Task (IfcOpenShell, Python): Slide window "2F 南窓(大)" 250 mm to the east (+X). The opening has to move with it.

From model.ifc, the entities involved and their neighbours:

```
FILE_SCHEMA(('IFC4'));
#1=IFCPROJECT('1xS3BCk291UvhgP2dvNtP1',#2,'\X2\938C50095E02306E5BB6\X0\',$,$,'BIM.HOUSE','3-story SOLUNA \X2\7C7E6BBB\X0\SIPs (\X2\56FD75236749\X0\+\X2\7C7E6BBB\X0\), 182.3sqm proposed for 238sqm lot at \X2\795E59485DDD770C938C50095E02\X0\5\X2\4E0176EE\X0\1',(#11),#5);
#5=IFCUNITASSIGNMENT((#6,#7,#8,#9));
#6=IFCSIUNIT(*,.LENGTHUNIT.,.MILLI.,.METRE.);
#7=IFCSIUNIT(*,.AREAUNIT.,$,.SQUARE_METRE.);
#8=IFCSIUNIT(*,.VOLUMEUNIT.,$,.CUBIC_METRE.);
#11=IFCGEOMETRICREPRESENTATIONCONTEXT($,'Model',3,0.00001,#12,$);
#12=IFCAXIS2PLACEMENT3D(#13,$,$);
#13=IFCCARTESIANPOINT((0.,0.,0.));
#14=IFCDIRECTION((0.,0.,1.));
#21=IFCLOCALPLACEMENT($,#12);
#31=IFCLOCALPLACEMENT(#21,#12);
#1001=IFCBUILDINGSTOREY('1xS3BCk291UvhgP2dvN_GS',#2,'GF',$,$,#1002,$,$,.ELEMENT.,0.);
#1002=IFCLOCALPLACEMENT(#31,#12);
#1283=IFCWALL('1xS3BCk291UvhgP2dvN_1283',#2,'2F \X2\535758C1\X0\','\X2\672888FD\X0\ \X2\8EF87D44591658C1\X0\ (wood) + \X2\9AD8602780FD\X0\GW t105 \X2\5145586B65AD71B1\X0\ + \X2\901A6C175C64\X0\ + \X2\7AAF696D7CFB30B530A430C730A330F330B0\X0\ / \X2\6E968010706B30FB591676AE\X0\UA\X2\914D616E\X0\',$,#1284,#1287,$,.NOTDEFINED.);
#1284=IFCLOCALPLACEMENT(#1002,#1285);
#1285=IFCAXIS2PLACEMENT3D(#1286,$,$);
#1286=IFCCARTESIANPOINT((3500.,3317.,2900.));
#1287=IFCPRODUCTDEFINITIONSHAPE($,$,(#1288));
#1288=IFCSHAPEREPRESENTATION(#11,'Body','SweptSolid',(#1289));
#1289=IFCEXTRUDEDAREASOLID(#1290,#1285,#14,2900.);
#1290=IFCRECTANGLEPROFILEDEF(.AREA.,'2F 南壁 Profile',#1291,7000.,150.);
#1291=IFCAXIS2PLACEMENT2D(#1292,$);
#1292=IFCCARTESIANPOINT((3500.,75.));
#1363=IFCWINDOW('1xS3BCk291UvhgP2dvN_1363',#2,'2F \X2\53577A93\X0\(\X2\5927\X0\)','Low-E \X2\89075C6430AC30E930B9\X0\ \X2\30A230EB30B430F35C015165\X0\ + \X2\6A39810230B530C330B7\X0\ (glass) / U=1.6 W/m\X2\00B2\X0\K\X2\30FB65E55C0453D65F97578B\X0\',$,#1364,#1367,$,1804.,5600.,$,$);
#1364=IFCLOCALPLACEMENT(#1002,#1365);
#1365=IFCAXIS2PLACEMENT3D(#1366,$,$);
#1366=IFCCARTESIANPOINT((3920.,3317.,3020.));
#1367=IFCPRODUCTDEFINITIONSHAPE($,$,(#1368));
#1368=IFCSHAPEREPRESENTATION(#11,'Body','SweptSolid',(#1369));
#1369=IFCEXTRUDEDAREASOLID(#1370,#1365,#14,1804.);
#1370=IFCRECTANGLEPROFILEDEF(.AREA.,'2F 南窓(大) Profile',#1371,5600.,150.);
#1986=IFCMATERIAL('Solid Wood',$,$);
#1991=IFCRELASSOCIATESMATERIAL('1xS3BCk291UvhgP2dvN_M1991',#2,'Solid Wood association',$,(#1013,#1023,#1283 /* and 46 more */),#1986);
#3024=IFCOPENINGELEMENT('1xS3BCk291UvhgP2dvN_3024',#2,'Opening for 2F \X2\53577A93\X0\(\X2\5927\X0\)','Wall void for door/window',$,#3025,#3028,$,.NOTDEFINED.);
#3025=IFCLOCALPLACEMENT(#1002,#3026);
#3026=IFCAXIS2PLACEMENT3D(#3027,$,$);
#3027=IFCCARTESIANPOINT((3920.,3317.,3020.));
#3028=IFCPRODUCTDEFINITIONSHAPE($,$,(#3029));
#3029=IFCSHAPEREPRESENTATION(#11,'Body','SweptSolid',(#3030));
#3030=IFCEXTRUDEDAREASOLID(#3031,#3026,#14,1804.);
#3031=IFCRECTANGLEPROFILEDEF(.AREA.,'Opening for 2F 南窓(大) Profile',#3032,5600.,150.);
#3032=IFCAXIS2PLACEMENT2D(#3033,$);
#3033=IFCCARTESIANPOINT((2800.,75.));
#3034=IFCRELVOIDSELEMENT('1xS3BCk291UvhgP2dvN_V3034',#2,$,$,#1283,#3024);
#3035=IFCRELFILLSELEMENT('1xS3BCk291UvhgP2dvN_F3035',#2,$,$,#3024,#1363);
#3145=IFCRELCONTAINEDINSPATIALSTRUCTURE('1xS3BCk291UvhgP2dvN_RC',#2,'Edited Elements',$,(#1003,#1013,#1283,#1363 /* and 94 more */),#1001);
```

```python
import ifcopenshell
import ifcopenshell.api.geometry
import ifcopenshell.util.placement

model = ifcopenshell.open("model.ifc")

window = model.by_guid("1xS3BCk291UvhgP2dvN_1363")
opening = window.FillsVoids[0].RelatingOpeningElement
wall = opening.VoidsElements[0].RelatingBuildingElement

wall_matrix = ifcopenshell.util.placement.get_local_placement(wall.ObjectPlacement)
shift = wall_matrix[:3, 0] * 250.0
before = ifcopenshell.util.placement.get_local_placement(window.ObjectPlacement)[:3, 3].copy()

# The window is not placed relative to its opening, so move both.
for product in (opening, window):
    matrix = ifcopenshell.util.placement.get_local_placement(product.ObjectPlacement)
    matrix[:3, 3] += shift
    ifcopenshell.api.geometry.edit_object_placement(model, product=product, matrix=matrix, is_si=False)

after = ifcopenshell.util.placement.get_local_placement(window.ObjectPlacement)[:3, 3]
print("window moved by", (after - before).round(3) + 0.0)

model.write("model_v2.ifc")
```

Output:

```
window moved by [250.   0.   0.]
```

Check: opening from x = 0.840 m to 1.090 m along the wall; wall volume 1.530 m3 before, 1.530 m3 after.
